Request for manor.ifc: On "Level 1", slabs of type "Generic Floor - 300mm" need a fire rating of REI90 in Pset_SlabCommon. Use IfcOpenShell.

First a look at what the model holds.

```python
import ifcopenshell
import ifcopenshell.util.element

model = ifcopenshell.open("manor.ifc")
print(model.schema)
storey = next(s for s in model.by_type("IfcBuildingStorey") if s.Name == "Level 1")
slabs = [e for e in ifcopenshell.util.element.get_decomposition(storey) if e.is_a("IfcSlab")]
seen = {}
for e in slabs:
    element_type = ifcopenshell.util.element.get_type(e)
    key = (element_type.Name if element_type != e and element_type else None, ifcopenshell.util.element.get_pset(e, "Pset_SlabCommon", "FireRating"))
    seen[key] = seen.get(key, 0) + 1
for (name, value), count in sorted(seen.items(), key=str):
    print(count, "x", name, "|", value)
```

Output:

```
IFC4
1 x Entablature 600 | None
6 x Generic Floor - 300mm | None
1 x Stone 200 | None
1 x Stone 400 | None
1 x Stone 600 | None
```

```python
import ifcopenshell
import ifcopenshell.api.pset
import ifcopenshell.util.element

model = ifcopenshell.open("manor.ifc")

storey = next(s for s in model.by_type("IfcBuildingStorey") if s.Name == "Level 1")
slabs = [e for e in ifcopenshell.util.element.get_decomposition(storey) if e.is_a("IfcSlab")]

count = 0
for e in slabs:
    element_type = ifcopenshell.util.element.get_type(e)
    if element_type in (None, e) or element_type.Name != "Generic Floor - 300mm":
        continue
    # add_pset returns the element's existing set when there is one.
    pset = ifcopenshell.api.pset.add_pset(model, product=e, name="Pset_SlabCommon")
    ifcopenshell.api.pset.edit_pset(model, pset=pset, properties={"FireRating": "REI90"})
    count += 1

print(count, "slabs updated")

model.write("manor_edited.ifc")
```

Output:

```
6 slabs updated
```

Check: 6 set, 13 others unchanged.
